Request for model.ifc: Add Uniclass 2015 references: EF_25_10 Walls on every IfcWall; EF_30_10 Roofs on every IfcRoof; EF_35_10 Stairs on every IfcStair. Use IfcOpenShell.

First a look at what the model holds.

```python
import ifcopenshell

model = ifcopenshell.open("model.ifc")
print(model.schema)
print("classifications:", [c.Name for c in model.by_type("IfcClassification")])
for ifc_class in ("IfcDoor", "IfcRoof", "IfcStair", "IfcWall", "IfcWindow"):
    print(ifc_class, len(model.by_type(ifc_class)))
```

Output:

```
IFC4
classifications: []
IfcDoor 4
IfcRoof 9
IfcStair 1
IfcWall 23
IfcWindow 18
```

```python
import ifcopenshell
import ifcopenshell.api.classification

model = ifcopenshell.open("model.ifc")

system = ifcopenshell.api.classification.add_classification(model, classification="Uniclass 2015")

codes = {
    "IfcWall": ("EF_25_10", "Walls"),
    "IfcRoof": ("EF_30_10", "Roofs"),
    "IfcStair": ("EF_35_10", "Stairs"),
}
for ifc_class, (code, name) in codes.items():
    products = model.by_type(ifc_class)
    ifcopenshell.api.classification.add_reference(
        model, products=products, classification=system, identification=code, name=name
    )
    print(code, len(products))

model.write("model_rev.ifc")
```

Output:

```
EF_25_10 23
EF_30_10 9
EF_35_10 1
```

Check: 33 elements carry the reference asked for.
